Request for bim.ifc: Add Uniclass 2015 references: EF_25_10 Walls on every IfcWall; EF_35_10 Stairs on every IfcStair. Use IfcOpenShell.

First a look at what the model holds.

```python
import ifcopenshell

model = ifcopenshell.open("bim.ifc")
print(model.schema)
print("classifications:", [c.Name for c in model.by_type("IfcClassification")])
for ifc_class in ("IfcDoor", "IfcRoof", "IfcStair", "IfcWall", "IfcWindow"):
    print(ifc_class, len(model.by_type(ifc_class)))
```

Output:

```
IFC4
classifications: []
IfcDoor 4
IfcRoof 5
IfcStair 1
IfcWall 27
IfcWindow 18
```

```python
import ifcopenshell
import ifcopenshell.api.classification

model = ifcopenshell.open("bim.ifc")

system = ifcopenshell.api.classification.add_classification(model, classification="Uniclass 2015")

codes = {
    "IfcWall": ("EF_25_10", "Walls"),
    "IfcStair": ("EF_35_10", "Stairs"),
}
for ifc_class, (code, name) in codes.items():
    products = model.by_type(ifc_class)
    ifcopenshell.api.classification.add_reference(
        model, products=products, classification=system, identification=code, name=name
    )
    print(code, len(products))

model.write("bim_rev.ifc")
```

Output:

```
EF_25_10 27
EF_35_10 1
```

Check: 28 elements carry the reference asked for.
